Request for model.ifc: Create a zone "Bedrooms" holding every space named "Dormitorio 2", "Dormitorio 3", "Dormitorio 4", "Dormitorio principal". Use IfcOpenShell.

First a look at what the model holds.

```python
import ifcopenshell

model = ifcopenshell.open("model.ifc")
print(model.schema)
seen = {}
for space in model.by_type("IfcSpace"):
    seen[space.LongName] = seen.get(space.LongName, 0) + 1
for name, count in sorted(seen.items(), key=str):
    print(count, "x", name)
print("zones:", [z.Name for z in model.by_type("IfcZone")][:20])
```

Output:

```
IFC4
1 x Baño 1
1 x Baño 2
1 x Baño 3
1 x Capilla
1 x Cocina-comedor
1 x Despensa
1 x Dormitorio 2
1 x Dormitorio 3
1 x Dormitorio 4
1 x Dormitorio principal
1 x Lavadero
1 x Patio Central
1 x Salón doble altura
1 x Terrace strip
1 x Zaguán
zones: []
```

```python
import ifcopenshell
import ifcopenshell.api.group
import ifcopenshell.api.root

model = ifcopenshell.open("model.ifc")

names = {"Dormitorio 2", "Dormitorio 3", "Dormitorio 4", "Dormitorio principal"}
spaces = [s for s in model.by_type("IfcSpace") if s.LongName in names]

zone = ifcopenshell.api.root.create_entity(model, ifc_class="IfcZone", name="Bedrooms")
ifcopenshell.api.group.assign_group(model, products=spaces, group=zone)
print(len(spaces), "spaces in", zone.Name)

model.write("model-out.ifc")
```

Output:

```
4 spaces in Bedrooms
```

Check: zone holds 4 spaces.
